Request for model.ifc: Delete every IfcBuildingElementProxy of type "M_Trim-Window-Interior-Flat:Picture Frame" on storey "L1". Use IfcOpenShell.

First a look at what the model holds.

```python
import ifcopenshell
import ifcopenshell.util.element

model = ifcopenshell.open("model.ifc")
print(model.schema)
storey = next(s for s in model.by_type("IfcBuildingStorey") if s.Name == "L1")
proxies = [e for e in ifcopenshell.util.element.get_decomposition(storey) if e.is_a("IfcBuildingElementProxy")]
seen = {}
for e in proxies:
    element_type = ifcopenshell.util.element.get_type(e)
    name = element_type.Name if element_type not in (None, e) else None
    seen[name] = seen.get(name, 0) + 1
for name, count in sorted(seen.items(), key=str):
    print(count, "x", name)
```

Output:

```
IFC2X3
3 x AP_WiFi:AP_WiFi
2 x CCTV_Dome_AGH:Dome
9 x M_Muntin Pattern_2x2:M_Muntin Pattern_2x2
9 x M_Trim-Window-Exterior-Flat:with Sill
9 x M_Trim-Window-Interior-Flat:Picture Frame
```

```python
import ifcopenshell
import ifcopenshell.api.root
import ifcopenshell.util.element

model = ifcopenshell.open("model.ifc")

storey = next(s for s in model.by_type("IfcBuildingStorey") if s.Name == "L1")
proxies = [e for e in ifcopenshell.util.element.get_decomposition(storey) if e.is_a("IfcBuildingElementProxy")]
targets = [e for e in proxies if (t := ifcopenshell.util.element.get_type(e)) not in (None, e) and t.Name == "M_Trim-Window-Interior-Flat:Picture Frame"]

for e in targets:
    ifcopenshell.api.root.remove_product(model, product=e)
print(len(targets), "removed")

model.write("model_v2.ifc")
```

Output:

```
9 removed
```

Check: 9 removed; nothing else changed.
